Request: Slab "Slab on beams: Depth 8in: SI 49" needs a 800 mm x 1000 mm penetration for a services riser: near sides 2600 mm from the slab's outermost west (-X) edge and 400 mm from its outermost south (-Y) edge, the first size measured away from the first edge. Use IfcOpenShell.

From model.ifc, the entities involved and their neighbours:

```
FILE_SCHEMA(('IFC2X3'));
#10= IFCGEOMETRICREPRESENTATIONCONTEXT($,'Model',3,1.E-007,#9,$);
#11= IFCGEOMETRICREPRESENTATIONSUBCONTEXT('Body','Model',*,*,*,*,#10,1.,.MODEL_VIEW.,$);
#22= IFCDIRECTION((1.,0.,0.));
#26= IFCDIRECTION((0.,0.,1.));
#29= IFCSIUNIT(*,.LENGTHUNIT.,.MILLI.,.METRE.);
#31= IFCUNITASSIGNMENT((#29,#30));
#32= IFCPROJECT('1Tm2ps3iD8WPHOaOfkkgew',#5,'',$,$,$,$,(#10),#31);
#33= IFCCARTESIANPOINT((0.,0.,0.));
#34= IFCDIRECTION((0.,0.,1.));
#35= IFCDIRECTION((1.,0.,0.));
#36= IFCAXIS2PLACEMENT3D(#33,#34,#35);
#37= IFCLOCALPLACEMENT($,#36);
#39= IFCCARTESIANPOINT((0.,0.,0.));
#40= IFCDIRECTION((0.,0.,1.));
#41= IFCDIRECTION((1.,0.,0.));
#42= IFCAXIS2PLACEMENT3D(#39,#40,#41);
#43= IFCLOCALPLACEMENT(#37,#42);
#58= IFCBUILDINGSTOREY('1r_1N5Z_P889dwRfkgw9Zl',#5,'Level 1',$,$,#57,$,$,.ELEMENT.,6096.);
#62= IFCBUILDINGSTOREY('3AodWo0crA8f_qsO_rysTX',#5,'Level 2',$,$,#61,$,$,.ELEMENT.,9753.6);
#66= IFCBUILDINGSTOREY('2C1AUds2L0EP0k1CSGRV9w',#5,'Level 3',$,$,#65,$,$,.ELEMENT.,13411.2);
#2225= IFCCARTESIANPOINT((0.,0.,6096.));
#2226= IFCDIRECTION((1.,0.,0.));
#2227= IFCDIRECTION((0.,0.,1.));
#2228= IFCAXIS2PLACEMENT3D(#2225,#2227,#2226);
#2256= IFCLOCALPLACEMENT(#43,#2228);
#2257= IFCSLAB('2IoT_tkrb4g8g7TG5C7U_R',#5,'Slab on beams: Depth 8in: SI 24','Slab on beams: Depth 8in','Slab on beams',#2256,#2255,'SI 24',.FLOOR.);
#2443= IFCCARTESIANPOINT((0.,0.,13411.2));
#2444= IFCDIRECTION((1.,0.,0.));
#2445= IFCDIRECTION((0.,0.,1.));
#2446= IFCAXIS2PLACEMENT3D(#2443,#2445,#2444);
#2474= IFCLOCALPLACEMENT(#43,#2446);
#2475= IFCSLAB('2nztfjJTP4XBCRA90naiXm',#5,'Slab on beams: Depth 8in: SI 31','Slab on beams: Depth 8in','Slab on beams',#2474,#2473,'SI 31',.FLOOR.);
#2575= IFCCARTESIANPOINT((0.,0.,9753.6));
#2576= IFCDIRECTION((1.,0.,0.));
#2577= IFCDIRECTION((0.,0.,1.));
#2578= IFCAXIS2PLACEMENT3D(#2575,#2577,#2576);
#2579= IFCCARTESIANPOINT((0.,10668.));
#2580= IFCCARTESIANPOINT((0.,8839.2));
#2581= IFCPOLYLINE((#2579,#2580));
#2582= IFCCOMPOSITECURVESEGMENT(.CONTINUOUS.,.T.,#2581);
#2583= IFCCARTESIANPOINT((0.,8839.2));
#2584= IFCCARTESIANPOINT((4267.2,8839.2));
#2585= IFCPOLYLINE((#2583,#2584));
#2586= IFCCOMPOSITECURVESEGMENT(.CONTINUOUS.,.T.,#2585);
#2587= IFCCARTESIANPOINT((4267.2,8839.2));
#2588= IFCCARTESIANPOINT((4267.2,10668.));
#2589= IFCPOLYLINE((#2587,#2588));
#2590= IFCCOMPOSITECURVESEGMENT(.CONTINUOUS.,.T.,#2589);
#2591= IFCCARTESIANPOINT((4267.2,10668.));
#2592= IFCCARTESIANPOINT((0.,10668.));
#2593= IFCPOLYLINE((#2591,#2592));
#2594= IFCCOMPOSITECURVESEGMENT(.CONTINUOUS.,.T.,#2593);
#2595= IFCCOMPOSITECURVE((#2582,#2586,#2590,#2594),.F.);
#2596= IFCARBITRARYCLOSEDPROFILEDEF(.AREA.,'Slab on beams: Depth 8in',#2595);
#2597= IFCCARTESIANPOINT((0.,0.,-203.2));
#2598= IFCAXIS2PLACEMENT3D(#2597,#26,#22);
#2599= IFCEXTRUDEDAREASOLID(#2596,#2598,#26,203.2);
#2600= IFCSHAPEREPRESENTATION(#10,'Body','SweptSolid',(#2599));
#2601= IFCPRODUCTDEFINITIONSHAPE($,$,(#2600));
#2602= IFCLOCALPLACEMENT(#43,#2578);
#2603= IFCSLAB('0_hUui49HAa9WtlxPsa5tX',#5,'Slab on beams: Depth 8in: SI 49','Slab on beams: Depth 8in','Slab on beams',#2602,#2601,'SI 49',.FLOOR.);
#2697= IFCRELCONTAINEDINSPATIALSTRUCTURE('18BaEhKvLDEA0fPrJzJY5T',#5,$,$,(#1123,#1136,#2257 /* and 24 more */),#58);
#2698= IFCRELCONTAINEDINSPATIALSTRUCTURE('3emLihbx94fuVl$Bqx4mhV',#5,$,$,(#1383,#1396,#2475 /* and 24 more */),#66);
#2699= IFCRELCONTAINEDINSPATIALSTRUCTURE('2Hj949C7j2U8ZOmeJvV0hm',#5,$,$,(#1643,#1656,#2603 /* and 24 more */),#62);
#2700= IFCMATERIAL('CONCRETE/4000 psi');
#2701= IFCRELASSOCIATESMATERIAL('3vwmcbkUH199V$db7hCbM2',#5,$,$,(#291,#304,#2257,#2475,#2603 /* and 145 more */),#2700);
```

```python
import numpy as np
import ifcopenshell
import ifcopenshell.api.feature
import ifcopenshell.api.geometry
import ifcopenshell.api.root
import ifcopenshell.geom
import ifcopenshell.util.placement
import ifcopenshell.util.representation
import ifcopenshell.util.shape
import ifcopenshell.util.unit

model = ifcopenshell.open("model.ifc")
unit_scale = ifcopenshell.util.unit.calculate_unit_scale(model)
settings = ifcopenshell.geom.settings()


def volume(element):
    """Net volume in cubic metres, openings subtracted."""
    shape = ifcopenshell.geom.create_shape(settings, element)
    return ifcopenshell.util.shape.get_volume(shape.geometry)


slab = model.by_guid("0_hUui49HAa9WtlxPsa5tX")
before = volume(slab)

# Extent in the slab's own axes, in metres. The edges named are its -X and -Y sides.
slab_shape = ifcopenshell.geom.create_shape(settings, slab)
vertices = ifcopenshell.util.shape.get_vertices(slab_shape.geometry)
x_min, y_min, bottom = vertices.min(axis=0)
top = vertices[:, 2].max()

opening = ifcopenshell.api.root.create_entity(model, ifc_class="IfcOpeningElement", name="Services riser opening")
context = ifcopenshell.util.representation.get_context(model, "Model", "Body", "MODEL_VIEW")
width, depth = 0.8, 1
outline = [(0.0, 0.0), (width, 0.0), (width, depth), (0.0, depth), (0.0, 0.0)]
# Overshoot both faces by 50 mm so the cut is clean.
shape = ifcopenshell.api.geometry.add_slab_representation(
    model, context=context, depth=top - bottom + 0.1, polyline=outline
)
ifcopenshell.api.geometry.assign_representation(model, product=opening, representation=shape)

matrix = ifcopenshell.util.placement.get_local_placement(slab.ObjectPlacement)
matrix[:, 3] = matrix @ np.append(np.array([x_min + 2.6, y_min + 0.4, bottom - 0.05]) / unit_scale, 1.0)
ifcopenshell.api.geometry.edit_object_placement(model, product=opening, matrix=matrix, is_si=False)
ifcopenshell.api.feature.add_feature(model, feature=opening, element=slab)

after = volume(slab)

print(f"slab volume {before:.3f} -> {after:.3f} m3")

model.write("model_v2.ifc")
```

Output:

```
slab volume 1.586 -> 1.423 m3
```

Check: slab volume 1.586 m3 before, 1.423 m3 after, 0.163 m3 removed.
